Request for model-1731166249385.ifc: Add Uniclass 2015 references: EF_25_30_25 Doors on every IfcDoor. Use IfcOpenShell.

First a look at what the model holds.

```python
import ifcopenshell

model = ifcopenshell.open("model-1731166249385.ifc")
print(model.schema)
print("classifications:", [c.Name for c in model.by_type("IfcClassification")])
for ifc_class in ("IfcDoor", "IfcRoof", "IfcStair", "IfcWall", "IfcWindow"):
    print(ifc_class, len(model.by_type(ifc_class)))
```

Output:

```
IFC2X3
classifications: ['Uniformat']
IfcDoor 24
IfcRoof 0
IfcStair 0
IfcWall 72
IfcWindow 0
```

```python
import ifcopenshell
import ifcopenshell.api.classification

model = ifcopenshell.open("model-1731166249385.ifc")

# IFC2X3 requires Source and Edition and has no link from the project to the system.
system = model.create_entity("IfcClassification", Source="NBS", Edition="2015", Name="Uniclass 2015")

codes = {
    "IfcDoor": ("EF_25_30_25", "Doors"),
}
for ifc_class, (code, name) in codes.items():
    products = model.by_type(ifc_class)
    ifcopenshell.api.classification.add_reference(
        model, products=products, classification=system, identification=code, name=name
    )
    print(code, len(products))

model.write("model-1731166249385_v2.ifc")
```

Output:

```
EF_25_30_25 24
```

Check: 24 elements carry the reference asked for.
